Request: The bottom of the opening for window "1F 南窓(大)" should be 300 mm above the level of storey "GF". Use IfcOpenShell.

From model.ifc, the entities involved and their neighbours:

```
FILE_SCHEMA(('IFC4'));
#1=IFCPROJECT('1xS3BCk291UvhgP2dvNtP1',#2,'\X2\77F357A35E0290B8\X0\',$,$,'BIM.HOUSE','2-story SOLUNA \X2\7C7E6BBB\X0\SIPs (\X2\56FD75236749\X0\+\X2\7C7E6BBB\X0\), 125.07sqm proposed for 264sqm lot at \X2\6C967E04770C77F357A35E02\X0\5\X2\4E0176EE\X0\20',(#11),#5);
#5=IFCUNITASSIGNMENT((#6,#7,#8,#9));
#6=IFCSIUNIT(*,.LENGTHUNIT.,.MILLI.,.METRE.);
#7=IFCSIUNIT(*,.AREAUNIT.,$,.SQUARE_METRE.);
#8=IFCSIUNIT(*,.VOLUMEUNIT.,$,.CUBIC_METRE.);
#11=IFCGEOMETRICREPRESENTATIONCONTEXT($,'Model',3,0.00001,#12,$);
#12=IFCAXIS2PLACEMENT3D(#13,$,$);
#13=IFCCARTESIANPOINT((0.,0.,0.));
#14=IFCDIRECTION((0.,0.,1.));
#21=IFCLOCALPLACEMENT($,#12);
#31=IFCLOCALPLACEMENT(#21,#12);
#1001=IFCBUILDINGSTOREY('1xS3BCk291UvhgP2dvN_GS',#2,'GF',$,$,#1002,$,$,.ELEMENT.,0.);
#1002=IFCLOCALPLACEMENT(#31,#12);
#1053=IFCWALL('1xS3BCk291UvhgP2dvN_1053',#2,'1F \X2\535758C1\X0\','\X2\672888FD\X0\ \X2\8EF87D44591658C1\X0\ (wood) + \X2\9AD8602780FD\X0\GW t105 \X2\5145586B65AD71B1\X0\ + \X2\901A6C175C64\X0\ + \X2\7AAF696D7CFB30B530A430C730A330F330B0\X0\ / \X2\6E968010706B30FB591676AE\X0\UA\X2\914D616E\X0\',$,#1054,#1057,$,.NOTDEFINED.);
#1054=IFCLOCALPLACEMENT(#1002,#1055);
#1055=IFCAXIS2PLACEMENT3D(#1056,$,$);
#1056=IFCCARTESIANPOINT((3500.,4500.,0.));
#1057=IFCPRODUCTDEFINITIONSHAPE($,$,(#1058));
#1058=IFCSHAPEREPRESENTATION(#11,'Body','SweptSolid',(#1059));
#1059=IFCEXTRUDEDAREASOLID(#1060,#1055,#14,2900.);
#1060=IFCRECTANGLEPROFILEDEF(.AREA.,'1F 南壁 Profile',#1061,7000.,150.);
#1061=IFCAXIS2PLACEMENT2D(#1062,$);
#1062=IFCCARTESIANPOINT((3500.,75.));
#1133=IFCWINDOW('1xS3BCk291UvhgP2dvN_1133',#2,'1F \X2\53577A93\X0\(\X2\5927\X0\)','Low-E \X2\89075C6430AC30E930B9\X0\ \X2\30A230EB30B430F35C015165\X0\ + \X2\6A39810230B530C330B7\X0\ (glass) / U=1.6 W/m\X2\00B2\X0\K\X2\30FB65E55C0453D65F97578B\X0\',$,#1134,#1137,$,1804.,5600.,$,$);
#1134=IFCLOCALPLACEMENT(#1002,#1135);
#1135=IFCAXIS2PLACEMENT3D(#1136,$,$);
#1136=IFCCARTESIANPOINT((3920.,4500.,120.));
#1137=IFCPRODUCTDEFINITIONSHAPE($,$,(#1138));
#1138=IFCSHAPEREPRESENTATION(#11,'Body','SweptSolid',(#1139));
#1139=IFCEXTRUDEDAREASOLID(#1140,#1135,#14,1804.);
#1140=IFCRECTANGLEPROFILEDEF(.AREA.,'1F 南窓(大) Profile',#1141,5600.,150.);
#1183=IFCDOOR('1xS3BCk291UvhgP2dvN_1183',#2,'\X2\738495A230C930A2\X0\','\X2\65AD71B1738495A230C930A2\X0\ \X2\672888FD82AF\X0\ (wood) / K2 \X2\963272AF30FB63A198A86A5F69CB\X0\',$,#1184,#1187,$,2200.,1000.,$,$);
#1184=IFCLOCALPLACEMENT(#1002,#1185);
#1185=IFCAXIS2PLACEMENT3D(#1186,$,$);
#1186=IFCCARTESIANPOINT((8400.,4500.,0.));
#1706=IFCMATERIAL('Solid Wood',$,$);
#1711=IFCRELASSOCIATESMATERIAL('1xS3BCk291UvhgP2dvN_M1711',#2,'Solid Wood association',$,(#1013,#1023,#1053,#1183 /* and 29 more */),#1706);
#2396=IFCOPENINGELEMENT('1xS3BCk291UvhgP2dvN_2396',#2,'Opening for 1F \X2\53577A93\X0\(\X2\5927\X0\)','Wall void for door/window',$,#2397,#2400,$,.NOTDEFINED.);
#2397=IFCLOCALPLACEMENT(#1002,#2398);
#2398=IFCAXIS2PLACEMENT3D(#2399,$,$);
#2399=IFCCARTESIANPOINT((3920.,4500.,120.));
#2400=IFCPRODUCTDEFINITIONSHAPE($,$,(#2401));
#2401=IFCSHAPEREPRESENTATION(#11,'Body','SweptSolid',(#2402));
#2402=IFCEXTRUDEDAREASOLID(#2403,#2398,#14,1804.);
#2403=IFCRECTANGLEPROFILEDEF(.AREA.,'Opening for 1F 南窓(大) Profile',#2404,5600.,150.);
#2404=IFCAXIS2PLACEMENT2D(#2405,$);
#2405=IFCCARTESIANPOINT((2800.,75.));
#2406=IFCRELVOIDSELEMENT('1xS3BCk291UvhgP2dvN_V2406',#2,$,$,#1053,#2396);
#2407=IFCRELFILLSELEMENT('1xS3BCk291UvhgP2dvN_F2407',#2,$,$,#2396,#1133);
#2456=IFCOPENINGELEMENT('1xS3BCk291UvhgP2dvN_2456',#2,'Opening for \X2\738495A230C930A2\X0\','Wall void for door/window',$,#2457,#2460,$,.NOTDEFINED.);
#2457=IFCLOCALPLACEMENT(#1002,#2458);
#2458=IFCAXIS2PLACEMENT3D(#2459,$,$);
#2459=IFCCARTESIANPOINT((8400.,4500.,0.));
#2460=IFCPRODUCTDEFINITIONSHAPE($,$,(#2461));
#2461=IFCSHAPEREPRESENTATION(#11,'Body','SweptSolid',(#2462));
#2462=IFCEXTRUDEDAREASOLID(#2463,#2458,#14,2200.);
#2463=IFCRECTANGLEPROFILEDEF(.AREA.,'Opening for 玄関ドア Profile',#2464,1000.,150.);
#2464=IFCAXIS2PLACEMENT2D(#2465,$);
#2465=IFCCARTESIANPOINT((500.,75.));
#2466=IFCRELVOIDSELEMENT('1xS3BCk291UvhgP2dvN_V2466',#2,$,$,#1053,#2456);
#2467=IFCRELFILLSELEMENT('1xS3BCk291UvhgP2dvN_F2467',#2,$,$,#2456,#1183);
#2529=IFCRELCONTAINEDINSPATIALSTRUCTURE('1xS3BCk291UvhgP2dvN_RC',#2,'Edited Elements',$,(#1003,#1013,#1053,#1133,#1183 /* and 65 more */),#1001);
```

```python
import numpy as np
import ifcopenshell
import ifcopenshell.api.geometry
import ifcopenshell.geom
import ifcopenshell.util.element
import ifcopenshell.util.placement
import ifcopenshell.util.shape
import ifcopenshell.util.unit

model = ifcopenshell.open("model.ifc")
unit_scale = ifcopenshell.util.unit.calculate_unit_scale(model)

window = model.by_guid("1xS3BCk291UvhgP2dvN_1133")
opening = window.FillsVoids[0].RelatingOpeningElement
storey = ifcopenshell.util.element.get_container(window, ifc_class="IfcBuildingStorey")
level = ifcopenshell.util.placement.get_local_placement(storey.ObjectPlacement)[2, 3]

# The opening's origin need not be at the sill, so measure its lowest point.
shape = ifcopenshell.geom.create_shape(ifcopenshell.geom.settings(), opening)
bottom = ifcopenshell.util.shape.get_shape_bottom_elevation(shape, shape.geometry) / unit_scale
dz = level + 0.3 / unit_scale - bottom

shift = np.array([0.0, 0.0, dz])
# The window is not placed relative to its opening, so move both.
for product in (opening, window):
    matrix = ifcopenshell.util.placement.get_local_placement(product.ObjectPlacement)
    matrix[:3, 3] += shift
    ifcopenshell.api.geometry.edit_object_placement(model, product=product, matrix=matrix, is_si=False)

print(f"moved by {dz * unit_scale:+.3f} m")

model.write("model_edited.ifc")
```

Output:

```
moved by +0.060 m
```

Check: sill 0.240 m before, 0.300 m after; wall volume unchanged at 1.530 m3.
